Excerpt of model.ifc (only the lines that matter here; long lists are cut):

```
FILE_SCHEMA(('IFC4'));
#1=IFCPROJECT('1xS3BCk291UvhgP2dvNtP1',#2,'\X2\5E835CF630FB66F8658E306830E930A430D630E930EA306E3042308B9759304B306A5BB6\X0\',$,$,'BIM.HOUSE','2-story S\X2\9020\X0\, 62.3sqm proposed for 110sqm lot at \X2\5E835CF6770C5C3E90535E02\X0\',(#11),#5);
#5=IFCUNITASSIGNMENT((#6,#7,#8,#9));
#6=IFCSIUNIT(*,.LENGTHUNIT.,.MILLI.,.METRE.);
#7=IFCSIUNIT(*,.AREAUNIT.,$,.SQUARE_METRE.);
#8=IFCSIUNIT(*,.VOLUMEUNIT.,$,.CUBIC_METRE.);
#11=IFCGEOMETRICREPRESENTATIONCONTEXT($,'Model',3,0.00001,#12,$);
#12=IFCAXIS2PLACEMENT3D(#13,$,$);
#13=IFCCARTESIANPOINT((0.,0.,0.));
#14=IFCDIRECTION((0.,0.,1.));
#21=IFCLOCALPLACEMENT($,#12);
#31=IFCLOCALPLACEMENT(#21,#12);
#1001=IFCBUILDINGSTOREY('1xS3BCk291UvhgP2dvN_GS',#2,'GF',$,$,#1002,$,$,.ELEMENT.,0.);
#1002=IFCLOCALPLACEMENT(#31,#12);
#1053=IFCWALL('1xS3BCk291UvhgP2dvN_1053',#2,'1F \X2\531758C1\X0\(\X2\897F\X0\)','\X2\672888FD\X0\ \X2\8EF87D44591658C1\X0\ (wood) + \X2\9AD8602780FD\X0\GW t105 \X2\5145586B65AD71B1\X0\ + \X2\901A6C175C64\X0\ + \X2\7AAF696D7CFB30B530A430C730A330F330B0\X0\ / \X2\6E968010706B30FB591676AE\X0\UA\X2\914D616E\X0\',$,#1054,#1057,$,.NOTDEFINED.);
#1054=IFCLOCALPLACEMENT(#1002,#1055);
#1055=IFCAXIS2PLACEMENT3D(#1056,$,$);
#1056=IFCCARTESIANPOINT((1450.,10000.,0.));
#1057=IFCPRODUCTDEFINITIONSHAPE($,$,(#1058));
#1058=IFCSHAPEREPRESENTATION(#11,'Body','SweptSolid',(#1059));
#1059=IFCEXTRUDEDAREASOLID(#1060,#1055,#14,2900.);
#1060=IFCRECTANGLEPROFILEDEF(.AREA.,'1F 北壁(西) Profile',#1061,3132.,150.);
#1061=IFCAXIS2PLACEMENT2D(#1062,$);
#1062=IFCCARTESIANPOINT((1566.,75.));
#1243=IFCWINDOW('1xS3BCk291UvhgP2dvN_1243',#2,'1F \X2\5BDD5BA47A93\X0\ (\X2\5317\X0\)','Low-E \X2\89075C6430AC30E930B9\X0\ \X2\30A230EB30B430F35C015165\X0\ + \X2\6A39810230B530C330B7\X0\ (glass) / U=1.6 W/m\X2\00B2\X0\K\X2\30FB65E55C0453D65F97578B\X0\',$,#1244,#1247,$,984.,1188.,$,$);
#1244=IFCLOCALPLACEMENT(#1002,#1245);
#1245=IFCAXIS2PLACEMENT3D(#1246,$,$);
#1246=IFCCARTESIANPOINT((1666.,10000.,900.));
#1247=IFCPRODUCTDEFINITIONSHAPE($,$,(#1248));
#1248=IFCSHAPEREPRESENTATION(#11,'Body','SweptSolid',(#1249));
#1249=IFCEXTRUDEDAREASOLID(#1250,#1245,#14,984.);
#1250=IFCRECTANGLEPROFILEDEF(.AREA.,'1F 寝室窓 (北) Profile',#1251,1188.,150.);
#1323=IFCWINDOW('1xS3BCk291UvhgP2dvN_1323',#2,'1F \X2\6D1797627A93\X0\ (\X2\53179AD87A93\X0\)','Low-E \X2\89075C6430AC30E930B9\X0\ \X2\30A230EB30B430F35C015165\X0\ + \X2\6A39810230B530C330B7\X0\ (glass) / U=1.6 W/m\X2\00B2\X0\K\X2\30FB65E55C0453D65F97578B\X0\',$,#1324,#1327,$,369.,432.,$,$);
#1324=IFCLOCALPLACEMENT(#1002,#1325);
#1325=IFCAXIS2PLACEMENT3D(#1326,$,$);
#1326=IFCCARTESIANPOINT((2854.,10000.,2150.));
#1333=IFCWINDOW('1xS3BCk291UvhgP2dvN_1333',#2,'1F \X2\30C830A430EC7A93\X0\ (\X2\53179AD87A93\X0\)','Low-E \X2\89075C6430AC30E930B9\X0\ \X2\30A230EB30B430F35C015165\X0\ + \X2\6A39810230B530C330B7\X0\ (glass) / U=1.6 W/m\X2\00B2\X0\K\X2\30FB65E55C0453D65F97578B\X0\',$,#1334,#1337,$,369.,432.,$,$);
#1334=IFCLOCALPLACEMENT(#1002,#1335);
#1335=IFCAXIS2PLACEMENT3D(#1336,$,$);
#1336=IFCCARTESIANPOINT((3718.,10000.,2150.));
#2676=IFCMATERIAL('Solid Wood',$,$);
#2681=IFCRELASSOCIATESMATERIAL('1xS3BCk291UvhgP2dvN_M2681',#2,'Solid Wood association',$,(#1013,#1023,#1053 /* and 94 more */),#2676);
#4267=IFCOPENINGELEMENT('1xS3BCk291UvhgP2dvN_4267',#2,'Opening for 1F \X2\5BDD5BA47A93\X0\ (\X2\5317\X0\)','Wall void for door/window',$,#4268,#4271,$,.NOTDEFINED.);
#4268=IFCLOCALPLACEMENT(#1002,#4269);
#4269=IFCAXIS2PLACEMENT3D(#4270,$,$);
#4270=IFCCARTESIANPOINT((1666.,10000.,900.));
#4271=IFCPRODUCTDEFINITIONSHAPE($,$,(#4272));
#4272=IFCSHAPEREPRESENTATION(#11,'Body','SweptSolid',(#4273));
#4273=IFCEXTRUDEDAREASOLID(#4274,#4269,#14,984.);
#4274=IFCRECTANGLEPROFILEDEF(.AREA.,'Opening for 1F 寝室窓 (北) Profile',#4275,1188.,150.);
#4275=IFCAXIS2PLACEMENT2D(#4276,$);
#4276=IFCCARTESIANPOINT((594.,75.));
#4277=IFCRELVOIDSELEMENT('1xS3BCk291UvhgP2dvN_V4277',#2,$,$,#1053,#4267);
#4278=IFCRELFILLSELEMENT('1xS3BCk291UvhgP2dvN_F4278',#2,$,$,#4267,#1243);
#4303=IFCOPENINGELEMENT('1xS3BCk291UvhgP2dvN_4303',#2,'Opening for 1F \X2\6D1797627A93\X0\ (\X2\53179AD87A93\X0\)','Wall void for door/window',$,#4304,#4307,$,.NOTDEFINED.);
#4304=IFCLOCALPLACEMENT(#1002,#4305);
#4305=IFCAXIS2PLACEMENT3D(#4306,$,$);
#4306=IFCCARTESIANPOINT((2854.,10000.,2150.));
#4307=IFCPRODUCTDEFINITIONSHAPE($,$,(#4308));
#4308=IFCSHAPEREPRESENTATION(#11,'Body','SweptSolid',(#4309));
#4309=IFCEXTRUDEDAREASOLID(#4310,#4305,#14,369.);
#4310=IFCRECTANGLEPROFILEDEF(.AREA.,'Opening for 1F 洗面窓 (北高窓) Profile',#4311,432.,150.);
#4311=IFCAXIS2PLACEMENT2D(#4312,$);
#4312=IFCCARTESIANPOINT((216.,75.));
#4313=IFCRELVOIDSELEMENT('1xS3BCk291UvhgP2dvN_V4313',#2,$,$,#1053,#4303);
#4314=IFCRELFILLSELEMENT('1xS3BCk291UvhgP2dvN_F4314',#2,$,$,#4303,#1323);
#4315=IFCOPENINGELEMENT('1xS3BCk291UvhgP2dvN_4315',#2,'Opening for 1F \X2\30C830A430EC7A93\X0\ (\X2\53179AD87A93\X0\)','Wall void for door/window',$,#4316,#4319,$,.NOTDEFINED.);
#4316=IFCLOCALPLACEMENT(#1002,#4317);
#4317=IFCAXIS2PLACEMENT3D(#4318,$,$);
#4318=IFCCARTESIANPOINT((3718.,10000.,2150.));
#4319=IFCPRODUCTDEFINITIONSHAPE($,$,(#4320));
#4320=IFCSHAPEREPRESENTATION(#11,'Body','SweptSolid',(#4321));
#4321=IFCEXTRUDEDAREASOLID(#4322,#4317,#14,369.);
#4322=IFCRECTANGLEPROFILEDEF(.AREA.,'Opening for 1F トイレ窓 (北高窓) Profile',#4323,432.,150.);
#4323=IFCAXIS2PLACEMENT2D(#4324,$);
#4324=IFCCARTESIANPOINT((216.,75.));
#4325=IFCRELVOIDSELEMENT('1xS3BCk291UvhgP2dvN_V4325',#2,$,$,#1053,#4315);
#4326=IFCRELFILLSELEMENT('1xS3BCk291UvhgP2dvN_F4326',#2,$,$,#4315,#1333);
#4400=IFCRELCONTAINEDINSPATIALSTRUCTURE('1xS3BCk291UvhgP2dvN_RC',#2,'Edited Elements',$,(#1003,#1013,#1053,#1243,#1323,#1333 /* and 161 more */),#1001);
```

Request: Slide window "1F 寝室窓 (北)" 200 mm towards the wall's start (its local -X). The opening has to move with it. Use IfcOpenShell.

```python
import ifcopenshell
import ifcopenshell.api.geometry
import ifcopenshell.util.placement

model = ifcopenshell.open("model.ifc")

window = model.by_guid("1xS3BCk291UvhgP2dvN_1243")
opening = window.FillsVoids[0].RelatingOpeningElement
wall = opening.VoidsElements[0].RelatingBuildingElement

wall_matrix = ifcopenshell.util.placement.get_local_placement(wall.ObjectPlacement)
shift = wall_matrix[:3, 0] * -200.0
before = ifcopenshell.util.placement.get_local_placement(window.ObjectPlacement)[:3, 3].copy()

# The window is not placed relative to its opening, so move both.
for product in (opening, window):
    matrix = ifcopenshell.util.placement.get_local_placement(product.ObjectPlacement)
    matrix[:3, 3] += shift
    ifcopenshell.api.geometry.edit_object_placement(model, product=product, matrix=matrix, is_si=False)

after = ifcopenshell.util.placement.get_local_placement(window.ObjectPlacement)[:3, 3]
print("window moved by", (after - before).round(3) + 0.0)

model.write("model_rev.ifc")
```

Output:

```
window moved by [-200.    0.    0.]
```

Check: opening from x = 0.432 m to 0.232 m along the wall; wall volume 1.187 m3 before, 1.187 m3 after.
